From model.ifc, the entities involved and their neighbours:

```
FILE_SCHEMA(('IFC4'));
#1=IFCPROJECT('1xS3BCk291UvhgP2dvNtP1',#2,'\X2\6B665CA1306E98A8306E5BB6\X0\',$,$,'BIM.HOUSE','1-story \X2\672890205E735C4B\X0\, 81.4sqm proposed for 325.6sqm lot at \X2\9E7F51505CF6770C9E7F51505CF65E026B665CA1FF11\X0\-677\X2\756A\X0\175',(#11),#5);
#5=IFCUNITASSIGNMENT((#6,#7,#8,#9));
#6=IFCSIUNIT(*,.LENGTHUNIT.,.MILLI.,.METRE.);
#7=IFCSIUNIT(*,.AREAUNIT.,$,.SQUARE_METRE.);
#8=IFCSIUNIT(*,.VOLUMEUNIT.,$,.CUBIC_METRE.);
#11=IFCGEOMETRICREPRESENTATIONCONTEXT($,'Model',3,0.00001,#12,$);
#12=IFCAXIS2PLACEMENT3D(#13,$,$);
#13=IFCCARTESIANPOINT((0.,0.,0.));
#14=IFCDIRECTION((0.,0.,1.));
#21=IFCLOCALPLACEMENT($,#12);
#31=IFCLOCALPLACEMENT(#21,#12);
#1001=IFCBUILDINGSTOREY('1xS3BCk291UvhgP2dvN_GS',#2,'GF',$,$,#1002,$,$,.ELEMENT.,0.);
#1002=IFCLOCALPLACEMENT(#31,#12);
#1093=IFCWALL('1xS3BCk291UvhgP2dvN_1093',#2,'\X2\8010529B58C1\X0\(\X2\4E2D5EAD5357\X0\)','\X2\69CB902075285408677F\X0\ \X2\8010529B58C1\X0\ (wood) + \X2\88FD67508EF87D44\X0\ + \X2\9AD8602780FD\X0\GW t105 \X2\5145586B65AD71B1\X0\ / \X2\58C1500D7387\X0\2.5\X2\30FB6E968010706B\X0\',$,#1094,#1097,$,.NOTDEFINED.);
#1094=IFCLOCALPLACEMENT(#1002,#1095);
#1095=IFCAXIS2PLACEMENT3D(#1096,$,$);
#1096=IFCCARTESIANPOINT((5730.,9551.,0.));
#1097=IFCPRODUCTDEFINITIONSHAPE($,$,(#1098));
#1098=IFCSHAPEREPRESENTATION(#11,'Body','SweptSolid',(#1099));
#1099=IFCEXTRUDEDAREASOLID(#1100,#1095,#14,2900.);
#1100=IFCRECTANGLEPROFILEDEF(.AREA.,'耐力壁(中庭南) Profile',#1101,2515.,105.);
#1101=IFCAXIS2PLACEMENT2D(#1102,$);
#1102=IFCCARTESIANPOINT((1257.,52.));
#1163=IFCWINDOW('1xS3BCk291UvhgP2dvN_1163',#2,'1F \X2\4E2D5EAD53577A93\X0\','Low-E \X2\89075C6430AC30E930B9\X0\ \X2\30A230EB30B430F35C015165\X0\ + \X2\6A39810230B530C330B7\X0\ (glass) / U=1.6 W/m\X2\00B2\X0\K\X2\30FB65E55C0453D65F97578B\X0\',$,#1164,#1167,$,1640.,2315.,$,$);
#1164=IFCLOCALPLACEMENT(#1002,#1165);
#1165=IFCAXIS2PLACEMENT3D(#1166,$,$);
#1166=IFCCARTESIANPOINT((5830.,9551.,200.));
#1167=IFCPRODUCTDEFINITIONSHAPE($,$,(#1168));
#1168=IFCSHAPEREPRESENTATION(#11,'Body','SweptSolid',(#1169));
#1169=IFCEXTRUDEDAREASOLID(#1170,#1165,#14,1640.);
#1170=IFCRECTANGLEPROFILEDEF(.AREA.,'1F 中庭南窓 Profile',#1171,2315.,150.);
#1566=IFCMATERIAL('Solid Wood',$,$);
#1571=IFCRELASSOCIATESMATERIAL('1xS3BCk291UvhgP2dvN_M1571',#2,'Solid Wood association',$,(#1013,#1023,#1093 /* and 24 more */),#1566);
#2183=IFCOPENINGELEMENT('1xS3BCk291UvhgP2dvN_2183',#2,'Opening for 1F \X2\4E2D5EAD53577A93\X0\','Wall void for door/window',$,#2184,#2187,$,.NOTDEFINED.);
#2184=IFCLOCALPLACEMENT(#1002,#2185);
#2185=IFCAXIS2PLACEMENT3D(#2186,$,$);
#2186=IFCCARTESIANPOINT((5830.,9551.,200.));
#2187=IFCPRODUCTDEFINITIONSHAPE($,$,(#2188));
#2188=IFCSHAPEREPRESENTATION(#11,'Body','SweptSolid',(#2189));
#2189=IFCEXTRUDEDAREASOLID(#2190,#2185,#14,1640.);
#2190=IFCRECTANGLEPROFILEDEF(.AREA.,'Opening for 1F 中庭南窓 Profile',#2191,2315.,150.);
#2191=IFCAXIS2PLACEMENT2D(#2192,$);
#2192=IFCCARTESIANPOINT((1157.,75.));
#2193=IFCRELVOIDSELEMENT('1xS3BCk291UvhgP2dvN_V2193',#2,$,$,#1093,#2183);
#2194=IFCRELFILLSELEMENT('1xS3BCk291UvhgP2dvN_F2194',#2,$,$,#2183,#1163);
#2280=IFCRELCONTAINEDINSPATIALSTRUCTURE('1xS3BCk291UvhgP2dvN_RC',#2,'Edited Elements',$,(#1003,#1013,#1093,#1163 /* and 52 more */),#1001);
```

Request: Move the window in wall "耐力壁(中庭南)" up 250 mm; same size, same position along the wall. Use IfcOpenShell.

```python
import numpy as np
import ifcopenshell
import ifcopenshell.api.geometry
import ifcopenshell.util.placement
import ifcopenshell.util.unit

model = ifcopenshell.open("model.ifc")
unit_scale = ifcopenshell.util.unit.calculate_unit_scale(model)

window = model.by_guid("1xS3BCk291UvhgP2dvN_1163")
opening = window.FillsVoids[0].RelatingOpeningElement
dz = 250.0

shift = np.array([0.0, 0.0, dz])
# The window is not placed relative to its opening, so move both.
for product in (opening, window):
    matrix = ifcopenshell.util.placement.get_local_placement(product.ObjectPlacement)
    matrix[:3, 3] += shift
    ifcopenshell.api.geometry.edit_object_placement(model, product=product, matrix=matrix, is_si=False)

print(f"moved by {dz * unit_scale:+.3f} m")

model.write("model_v2.ifc")
```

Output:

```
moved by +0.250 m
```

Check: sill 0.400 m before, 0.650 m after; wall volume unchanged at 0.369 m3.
